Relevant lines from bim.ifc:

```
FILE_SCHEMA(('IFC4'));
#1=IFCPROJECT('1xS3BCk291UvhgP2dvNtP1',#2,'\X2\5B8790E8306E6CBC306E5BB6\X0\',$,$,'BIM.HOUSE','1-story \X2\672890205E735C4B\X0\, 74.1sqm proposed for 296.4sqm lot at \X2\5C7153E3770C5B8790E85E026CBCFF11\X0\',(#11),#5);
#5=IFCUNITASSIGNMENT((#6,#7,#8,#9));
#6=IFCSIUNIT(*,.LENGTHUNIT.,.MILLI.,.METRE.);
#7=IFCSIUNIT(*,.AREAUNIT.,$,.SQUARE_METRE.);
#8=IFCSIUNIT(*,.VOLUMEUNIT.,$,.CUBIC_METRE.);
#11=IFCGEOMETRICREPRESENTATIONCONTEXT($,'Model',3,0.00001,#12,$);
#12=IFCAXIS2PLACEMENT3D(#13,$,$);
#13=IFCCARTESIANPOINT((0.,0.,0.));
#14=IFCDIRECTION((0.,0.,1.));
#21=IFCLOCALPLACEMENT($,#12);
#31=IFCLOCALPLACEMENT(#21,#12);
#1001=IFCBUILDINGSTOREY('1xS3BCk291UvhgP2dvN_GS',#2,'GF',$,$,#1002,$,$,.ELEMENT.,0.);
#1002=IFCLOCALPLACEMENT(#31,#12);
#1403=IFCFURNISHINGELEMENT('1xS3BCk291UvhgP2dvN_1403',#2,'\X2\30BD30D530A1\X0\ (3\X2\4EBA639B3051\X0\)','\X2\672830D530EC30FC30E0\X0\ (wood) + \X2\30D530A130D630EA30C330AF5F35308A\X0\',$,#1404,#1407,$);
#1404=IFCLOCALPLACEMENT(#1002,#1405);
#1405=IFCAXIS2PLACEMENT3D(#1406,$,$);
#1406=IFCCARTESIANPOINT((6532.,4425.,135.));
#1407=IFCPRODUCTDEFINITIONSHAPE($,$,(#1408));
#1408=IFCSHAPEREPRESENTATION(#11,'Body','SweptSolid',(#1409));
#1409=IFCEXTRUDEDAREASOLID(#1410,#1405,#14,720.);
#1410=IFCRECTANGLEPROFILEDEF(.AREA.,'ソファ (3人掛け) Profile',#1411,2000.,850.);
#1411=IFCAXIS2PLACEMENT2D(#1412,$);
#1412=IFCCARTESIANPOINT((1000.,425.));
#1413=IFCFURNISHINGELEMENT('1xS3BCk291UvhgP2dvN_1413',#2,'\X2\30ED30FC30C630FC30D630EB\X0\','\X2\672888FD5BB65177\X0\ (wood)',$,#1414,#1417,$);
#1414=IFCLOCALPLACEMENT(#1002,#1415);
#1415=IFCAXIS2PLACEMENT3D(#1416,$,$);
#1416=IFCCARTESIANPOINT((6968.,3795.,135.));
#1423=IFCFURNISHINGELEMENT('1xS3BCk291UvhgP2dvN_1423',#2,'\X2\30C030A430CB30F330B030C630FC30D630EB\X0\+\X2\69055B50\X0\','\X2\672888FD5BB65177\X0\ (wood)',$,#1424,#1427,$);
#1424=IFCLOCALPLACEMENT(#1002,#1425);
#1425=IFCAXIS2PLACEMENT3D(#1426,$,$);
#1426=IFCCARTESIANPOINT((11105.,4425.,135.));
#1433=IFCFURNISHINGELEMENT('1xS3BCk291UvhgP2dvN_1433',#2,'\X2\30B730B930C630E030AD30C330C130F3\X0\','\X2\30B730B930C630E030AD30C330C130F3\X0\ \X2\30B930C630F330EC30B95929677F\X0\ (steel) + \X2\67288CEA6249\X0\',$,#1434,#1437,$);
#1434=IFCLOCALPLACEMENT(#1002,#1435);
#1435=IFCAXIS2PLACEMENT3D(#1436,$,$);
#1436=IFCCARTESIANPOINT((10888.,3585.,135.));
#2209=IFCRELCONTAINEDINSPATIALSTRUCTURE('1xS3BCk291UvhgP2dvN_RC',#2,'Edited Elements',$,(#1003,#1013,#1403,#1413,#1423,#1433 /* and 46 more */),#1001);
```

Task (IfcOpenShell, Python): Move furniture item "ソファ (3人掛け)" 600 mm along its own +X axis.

```python
import ifcopenshell
import ifcopenshell.api.geometry
import ifcopenshell.util.placement
import ifcopenshell.util.unit

model = ifcopenshell.open("bim.ifc")
unit_scale = ifcopenshell.util.unit.calculate_unit_scale(model)

item = model.by_guid("1xS3BCk291UvhgP2dvN_1403")
matrix = ifcopenshell.util.placement.get_local_placement(item.ObjectPlacement)
matrix[:3, 3] += matrix[:3, 0] * 0.6 / unit_scale
ifcopenshell.api.geometry.edit_object_placement(model, product=item, matrix=matrix, is_si=False)

print(ifcopenshell.util.placement.get_local_placement(item.ObjectPlacement).round(3) + 0.0)

model.write("bim_v2.ifc")
```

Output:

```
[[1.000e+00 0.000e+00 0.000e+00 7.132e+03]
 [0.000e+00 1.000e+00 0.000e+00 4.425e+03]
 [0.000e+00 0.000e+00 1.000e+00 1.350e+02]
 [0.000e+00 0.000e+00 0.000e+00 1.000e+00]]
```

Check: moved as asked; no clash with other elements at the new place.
